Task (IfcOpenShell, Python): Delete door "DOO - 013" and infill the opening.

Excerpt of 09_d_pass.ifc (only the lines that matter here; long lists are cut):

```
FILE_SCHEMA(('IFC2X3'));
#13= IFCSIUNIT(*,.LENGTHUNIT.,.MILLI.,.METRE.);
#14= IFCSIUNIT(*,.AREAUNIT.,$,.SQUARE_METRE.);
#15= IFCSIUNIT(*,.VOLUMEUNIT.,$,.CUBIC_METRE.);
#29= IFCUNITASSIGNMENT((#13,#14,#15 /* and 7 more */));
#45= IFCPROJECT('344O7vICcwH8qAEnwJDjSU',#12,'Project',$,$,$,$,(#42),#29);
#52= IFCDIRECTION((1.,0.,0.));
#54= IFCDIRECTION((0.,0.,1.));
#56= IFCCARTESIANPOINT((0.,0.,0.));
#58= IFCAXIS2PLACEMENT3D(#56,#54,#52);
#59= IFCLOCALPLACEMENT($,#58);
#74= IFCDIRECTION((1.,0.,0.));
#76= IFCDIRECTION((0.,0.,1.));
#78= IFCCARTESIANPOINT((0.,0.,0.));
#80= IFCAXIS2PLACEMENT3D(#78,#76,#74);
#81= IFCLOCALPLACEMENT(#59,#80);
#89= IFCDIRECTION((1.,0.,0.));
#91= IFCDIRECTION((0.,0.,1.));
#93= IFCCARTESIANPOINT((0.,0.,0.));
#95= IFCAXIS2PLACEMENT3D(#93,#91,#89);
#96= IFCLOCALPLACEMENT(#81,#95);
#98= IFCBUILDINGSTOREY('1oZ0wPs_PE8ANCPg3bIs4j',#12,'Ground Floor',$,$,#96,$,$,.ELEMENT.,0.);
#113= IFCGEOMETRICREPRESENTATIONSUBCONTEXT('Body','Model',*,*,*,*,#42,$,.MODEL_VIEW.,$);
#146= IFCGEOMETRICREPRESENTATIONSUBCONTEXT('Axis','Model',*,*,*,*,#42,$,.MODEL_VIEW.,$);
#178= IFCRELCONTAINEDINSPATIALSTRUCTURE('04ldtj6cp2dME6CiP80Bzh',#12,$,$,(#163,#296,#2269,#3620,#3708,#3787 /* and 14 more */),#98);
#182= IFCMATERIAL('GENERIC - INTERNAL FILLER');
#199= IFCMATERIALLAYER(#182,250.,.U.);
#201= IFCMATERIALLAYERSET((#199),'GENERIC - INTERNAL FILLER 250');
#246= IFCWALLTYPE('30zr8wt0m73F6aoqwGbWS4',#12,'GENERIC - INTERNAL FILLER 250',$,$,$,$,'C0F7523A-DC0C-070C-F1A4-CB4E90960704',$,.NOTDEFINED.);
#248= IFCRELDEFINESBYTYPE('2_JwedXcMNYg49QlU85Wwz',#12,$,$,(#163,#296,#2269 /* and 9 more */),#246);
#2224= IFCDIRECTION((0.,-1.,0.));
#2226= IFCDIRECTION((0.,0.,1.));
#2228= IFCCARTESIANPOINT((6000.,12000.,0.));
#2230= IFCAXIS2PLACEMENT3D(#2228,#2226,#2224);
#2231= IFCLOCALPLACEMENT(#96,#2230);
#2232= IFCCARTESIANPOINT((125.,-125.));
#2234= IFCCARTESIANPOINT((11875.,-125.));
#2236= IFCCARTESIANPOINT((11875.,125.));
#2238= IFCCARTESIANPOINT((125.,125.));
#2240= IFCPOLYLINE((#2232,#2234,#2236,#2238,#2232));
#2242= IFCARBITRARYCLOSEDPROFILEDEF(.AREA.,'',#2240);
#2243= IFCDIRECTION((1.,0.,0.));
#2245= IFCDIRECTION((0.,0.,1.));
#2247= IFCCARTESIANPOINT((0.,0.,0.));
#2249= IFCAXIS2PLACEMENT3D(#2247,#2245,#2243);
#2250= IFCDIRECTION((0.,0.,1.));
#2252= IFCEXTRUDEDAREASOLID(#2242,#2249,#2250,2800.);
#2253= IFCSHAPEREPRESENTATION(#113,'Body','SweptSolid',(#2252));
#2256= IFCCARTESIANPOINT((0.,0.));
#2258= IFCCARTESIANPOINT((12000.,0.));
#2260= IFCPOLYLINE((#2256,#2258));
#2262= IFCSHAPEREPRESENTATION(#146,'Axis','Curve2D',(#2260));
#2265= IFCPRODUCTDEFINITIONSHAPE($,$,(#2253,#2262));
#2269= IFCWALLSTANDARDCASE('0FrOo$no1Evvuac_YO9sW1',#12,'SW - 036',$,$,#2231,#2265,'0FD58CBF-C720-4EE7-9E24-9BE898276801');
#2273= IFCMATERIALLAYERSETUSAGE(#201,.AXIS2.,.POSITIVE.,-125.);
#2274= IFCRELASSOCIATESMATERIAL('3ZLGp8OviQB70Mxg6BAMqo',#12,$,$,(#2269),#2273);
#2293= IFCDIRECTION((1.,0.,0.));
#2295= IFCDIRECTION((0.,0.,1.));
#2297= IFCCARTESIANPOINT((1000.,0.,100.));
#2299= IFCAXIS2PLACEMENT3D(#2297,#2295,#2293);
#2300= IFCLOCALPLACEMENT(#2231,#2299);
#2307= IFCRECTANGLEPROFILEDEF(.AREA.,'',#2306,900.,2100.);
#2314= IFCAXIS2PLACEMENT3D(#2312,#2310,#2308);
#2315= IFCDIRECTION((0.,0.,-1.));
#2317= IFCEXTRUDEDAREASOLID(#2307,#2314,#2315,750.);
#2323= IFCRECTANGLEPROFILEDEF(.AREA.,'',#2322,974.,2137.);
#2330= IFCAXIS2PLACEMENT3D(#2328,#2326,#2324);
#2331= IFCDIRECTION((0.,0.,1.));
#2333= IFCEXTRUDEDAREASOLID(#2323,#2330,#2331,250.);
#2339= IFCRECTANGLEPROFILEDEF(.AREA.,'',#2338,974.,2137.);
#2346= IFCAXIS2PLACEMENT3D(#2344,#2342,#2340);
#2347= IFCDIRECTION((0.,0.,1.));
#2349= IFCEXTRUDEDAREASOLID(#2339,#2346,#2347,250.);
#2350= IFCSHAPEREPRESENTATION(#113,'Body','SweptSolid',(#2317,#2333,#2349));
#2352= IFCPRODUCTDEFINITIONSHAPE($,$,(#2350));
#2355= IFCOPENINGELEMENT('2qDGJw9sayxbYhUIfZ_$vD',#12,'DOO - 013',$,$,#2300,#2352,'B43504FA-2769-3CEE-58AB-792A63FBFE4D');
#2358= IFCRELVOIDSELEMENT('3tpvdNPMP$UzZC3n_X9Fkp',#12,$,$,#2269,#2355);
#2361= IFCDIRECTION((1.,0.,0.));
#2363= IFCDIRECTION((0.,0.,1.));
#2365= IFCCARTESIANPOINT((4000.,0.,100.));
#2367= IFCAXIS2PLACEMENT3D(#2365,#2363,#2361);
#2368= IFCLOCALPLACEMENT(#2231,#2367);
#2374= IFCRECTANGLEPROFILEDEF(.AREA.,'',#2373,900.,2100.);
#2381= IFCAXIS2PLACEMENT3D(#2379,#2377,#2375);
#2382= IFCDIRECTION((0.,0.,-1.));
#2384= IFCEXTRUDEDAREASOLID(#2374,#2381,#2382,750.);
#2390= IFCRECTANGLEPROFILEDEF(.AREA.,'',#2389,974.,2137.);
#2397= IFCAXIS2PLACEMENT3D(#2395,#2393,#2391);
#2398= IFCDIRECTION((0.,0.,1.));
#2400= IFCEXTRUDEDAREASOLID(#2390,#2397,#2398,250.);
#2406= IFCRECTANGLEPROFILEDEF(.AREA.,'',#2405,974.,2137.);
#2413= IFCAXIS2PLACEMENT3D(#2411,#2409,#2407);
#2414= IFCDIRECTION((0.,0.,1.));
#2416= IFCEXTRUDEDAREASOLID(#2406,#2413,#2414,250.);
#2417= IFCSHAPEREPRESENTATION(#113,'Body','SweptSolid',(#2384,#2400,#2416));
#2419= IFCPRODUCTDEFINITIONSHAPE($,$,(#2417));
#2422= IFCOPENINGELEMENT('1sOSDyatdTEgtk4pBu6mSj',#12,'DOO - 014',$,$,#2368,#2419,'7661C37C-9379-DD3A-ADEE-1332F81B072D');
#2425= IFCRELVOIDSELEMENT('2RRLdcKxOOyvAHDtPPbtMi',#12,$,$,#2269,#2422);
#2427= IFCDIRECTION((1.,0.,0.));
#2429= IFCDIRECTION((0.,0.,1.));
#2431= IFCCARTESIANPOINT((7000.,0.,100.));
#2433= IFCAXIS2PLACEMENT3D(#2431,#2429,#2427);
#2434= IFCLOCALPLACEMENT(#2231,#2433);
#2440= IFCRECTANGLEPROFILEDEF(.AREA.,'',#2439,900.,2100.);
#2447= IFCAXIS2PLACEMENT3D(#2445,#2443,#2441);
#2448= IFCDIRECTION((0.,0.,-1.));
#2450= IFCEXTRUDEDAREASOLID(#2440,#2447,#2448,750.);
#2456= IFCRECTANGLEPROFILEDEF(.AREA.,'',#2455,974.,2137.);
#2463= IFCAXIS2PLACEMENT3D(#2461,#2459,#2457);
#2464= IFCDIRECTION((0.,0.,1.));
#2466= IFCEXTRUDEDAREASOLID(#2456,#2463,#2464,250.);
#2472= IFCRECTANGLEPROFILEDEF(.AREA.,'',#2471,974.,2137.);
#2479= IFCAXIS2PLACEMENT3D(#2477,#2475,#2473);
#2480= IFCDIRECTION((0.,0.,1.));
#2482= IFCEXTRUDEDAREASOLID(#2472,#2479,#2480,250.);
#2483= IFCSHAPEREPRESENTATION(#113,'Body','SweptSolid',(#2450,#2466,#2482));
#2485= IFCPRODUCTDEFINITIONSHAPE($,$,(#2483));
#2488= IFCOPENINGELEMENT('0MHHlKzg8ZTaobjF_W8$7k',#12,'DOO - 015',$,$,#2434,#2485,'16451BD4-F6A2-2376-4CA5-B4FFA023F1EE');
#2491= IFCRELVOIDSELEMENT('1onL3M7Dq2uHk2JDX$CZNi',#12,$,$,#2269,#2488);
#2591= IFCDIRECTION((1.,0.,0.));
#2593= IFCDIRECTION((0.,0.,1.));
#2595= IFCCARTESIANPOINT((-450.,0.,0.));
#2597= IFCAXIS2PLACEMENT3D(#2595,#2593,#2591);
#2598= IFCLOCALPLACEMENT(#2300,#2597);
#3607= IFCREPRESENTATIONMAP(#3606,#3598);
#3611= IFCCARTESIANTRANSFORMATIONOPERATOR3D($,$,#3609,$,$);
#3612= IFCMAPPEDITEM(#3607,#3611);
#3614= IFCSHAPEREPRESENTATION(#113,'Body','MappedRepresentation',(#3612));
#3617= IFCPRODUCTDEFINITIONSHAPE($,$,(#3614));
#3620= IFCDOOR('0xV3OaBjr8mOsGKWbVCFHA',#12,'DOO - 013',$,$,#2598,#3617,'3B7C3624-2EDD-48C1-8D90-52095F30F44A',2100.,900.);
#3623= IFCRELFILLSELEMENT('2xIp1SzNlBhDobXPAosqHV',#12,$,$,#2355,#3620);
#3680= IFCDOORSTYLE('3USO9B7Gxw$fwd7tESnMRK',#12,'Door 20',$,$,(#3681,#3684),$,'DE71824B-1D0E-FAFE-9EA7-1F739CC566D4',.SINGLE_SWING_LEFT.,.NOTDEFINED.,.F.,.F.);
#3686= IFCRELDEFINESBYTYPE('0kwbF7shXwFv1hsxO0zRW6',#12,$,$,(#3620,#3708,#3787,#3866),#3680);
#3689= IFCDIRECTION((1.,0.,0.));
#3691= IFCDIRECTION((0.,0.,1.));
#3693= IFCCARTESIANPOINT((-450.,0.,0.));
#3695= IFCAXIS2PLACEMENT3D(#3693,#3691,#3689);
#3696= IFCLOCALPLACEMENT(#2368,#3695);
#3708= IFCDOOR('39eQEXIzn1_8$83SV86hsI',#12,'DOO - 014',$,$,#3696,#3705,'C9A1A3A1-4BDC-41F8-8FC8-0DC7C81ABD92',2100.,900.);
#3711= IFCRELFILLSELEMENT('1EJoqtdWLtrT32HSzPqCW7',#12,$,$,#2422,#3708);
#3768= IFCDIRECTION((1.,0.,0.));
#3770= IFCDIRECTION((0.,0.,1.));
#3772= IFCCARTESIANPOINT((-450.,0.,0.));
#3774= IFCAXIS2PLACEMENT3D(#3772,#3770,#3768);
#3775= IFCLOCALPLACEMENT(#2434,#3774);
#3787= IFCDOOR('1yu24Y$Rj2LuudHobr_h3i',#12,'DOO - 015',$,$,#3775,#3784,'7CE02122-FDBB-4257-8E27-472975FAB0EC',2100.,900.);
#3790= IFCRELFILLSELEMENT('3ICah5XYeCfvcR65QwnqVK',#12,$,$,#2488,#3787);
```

```python
import ifcopenshell
import ifcopenshell.api.feature
import ifcopenshell.api.root
import ifcopenshell.geom
import ifcopenshell.util.shape

model = ifcopenshell.open("09_d_pass.ifc")
settings = ifcopenshell.geom.settings()


def volume(element):
    """Net volume in cubic metres, openings subtracted."""
    shape = ifcopenshell.geom.create_shape(settings, element)
    return ifcopenshell.util.shape.get_volume(shape.geometry)


door = model.by_id(3620)
opening = door.FillsVoids[0].RelatingOpeningElement
wall = opening.VoidsElements[0].RelatingBuildingElement
before = volume(wall)

ifcopenshell.api.root.remove_product(model, product=door)
ifcopenshell.api.feature.remove_feature(model, feature=opening)

after = volume(wall)

print(f"wall volume {before:.3f} -> {after:.3f} m3")

model.write("09_d_pass_edited.ifc")
```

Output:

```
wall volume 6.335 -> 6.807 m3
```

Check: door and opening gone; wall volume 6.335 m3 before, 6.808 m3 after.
